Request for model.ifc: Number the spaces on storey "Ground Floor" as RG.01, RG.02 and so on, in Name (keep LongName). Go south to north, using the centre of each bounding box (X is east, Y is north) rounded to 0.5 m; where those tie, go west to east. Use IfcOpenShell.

First a look at what the model holds.

```python
import ifcopenshell
import ifcopenshell.util.element
import ifcopenshell.util.placement

model = ifcopenshell.open("model.ifc")
print(model.schema)
storey = next(s for s in model.by_type("IfcBuildingStorey") if s.Name == "Ground Floor")
spaces = [e for e in ifcopenshell.util.element.get_decomposition(storey) if e.is_a("IfcSpace")]
for e in sorted(spaces, key=lambda e: e.id()):
    origin = ifcopenshell.util.placement.get_local_placement(e.ObjectPlacement)[:3, 3]
    print(e.id(), e.Name, e.LongName, origin.round(2) + 0.0, sep=" | ")
```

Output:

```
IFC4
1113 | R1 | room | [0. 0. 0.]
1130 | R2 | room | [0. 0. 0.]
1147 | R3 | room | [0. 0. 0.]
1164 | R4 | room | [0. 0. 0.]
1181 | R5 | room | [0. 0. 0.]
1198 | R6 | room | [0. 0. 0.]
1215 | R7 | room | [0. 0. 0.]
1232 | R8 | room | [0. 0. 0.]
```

```python
import ifcopenshell
import ifcopenshell.geom
import ifcopenshell.util.element
import ifcopenshell.util.shape

model = ifcopenshell.open("model.ifc")
settings = ifcopenshell.geom.settings()
settings.set("use-world-coords", True)


def centre(element):
    shape = ifcopenshell.geom.create_shape(settings, element)
    return ifcopenshell.util.shape.get_bbox_centroid(shape.geometry)


storey = next(s for s in model.by_type("IfcBuildingStorey") if s.Name == "Ground Floor")
spaces = [e for e in ifcopenshell.util.element.get_decomposition(storey) if e.is_a("IfcSpace")]

# Insertion points can sit at a corner or the storey origin, so sort by the geometry (in metres).
centres = {e: centre(e) for e in spaces}
spaces.sort(key=lambda e: (round(centres[e][1] / 0.5), centres[e][0]))

for i, e in enumerate(spaces, start=1):
    number = f"RG.{i:02d}"
    e.Name = number
    print(e.id(), number)

model.write("model_updated.ifc")
```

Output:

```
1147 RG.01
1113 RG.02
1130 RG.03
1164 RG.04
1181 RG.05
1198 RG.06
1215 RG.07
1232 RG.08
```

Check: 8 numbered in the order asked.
